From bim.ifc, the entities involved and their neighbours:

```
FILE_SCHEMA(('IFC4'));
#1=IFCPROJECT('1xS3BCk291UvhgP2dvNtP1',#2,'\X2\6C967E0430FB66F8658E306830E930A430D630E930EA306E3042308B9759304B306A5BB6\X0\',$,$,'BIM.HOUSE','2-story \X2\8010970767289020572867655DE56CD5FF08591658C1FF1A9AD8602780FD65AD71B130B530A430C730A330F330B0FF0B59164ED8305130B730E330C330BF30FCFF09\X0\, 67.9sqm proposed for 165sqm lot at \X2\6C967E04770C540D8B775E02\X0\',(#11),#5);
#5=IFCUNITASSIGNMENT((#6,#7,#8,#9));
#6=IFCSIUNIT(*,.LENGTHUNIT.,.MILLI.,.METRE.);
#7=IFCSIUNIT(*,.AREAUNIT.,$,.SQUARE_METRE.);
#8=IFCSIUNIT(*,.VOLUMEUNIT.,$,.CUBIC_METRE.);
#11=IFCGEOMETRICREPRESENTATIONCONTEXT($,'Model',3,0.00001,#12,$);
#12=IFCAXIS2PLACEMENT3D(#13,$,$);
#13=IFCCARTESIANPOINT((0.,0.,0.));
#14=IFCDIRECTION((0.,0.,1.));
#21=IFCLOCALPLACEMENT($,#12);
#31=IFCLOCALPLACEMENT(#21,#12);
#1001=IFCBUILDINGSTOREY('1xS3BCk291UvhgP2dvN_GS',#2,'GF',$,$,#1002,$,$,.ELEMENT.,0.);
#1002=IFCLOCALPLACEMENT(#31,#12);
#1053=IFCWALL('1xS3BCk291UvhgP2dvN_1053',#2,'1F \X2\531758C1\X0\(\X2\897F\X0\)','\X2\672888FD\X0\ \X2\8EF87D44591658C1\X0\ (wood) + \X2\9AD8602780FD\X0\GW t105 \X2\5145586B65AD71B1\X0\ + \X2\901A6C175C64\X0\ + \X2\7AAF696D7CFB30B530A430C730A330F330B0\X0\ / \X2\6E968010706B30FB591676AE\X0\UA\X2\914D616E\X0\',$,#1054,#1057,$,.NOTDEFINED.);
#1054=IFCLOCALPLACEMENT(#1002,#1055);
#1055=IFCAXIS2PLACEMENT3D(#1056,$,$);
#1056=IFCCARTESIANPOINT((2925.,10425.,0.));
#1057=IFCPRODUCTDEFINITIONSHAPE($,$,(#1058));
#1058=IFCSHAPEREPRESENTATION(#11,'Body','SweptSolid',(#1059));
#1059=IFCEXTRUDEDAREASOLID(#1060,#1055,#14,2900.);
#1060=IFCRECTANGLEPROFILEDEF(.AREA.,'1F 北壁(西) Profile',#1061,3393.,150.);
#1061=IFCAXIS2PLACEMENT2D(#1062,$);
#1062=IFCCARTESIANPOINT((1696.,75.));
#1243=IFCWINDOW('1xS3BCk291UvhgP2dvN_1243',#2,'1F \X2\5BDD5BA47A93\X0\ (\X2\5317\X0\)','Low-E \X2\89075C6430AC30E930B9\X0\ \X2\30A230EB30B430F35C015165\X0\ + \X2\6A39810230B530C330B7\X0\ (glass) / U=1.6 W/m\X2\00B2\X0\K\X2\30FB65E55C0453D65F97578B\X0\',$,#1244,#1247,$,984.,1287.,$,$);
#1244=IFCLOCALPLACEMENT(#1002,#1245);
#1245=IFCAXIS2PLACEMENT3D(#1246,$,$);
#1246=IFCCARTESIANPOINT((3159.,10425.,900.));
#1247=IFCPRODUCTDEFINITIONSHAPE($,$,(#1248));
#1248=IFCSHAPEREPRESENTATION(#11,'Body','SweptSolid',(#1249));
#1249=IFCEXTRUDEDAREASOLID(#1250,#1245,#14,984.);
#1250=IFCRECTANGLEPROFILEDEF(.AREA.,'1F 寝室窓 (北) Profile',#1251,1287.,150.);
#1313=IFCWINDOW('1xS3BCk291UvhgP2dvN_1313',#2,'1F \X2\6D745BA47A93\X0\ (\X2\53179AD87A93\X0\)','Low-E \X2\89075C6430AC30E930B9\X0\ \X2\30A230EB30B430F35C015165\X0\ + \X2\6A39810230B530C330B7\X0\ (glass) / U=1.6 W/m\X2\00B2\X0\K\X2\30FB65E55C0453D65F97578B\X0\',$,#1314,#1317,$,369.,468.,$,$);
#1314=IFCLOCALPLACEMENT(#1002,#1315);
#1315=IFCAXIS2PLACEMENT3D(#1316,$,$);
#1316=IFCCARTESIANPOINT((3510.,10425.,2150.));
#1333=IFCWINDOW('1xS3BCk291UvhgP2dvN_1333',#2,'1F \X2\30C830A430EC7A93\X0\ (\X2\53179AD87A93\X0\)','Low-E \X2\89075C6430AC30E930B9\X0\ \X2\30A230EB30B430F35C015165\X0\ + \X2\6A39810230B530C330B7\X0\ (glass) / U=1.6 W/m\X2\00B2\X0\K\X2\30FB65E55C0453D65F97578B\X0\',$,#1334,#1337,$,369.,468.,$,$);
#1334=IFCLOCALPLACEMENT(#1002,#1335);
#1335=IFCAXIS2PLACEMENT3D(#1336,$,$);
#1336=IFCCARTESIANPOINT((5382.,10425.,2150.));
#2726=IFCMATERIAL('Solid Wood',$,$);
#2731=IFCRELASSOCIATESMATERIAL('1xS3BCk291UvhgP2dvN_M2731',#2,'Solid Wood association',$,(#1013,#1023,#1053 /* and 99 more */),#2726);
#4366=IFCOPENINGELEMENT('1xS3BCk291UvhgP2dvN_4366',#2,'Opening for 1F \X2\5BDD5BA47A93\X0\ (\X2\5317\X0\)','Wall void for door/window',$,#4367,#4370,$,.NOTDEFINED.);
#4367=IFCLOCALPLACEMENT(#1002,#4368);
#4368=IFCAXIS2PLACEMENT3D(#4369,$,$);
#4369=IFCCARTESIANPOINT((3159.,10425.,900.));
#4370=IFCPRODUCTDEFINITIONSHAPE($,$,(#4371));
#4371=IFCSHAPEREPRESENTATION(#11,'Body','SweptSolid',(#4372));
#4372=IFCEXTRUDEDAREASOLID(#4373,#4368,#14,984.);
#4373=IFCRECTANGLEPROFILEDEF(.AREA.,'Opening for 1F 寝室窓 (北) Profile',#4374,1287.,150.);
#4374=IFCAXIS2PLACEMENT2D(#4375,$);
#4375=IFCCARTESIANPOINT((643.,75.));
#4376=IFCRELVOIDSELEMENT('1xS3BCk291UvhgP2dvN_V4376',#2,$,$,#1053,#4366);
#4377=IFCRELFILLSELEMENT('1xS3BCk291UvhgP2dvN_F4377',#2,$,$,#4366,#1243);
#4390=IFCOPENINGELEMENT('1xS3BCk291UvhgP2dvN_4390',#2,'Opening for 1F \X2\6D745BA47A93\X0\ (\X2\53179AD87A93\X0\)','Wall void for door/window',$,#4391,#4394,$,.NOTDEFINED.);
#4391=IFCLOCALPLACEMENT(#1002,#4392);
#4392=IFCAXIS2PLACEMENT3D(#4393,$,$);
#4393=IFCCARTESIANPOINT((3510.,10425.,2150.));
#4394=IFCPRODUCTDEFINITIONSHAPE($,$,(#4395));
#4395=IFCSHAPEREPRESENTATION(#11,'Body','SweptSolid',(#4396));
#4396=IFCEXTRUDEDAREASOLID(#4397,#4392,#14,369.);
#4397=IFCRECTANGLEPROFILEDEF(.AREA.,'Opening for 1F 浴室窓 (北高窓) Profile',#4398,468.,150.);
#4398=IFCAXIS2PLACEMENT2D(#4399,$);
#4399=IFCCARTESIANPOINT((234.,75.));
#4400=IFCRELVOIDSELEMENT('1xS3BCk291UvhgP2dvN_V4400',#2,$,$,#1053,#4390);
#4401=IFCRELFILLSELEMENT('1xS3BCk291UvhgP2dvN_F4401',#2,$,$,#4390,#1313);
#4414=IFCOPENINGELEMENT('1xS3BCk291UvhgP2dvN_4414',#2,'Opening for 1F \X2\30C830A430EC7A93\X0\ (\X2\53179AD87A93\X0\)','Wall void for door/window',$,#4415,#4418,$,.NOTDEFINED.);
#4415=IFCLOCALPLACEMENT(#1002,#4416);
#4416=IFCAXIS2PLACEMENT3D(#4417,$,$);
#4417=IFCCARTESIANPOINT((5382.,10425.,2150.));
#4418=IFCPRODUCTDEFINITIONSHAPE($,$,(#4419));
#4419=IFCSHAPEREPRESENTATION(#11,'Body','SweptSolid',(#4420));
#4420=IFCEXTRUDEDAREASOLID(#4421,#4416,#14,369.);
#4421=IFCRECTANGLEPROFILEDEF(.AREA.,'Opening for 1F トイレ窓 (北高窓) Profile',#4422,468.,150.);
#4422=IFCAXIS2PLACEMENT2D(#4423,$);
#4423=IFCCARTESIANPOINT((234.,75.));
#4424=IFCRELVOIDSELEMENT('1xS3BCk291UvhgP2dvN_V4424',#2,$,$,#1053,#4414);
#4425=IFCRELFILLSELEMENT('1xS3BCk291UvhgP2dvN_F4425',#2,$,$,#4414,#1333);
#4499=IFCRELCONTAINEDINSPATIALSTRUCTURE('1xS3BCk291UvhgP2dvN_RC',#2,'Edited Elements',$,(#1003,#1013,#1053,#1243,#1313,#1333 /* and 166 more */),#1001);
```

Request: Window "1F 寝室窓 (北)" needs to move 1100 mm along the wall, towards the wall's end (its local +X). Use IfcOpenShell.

```python
import ifcopenshell
import ifcopenshell.api.geometry
import ifcopenshell.util.placement
import ifcopenshell.util.unit

model = ifcopenshell.open("bim.ifc")
unit_scale = ifcopenshell.util.unit.calculate_unit_scale(model)

window = model.by_id(1243)
opening = window.FillsVoids[0].RelatingOpeningElement
wall = opening.VoidsElements[0].RelatingBuildingElement

wall_matrix = ifcopenshell.util.placement.get_local_placement(wall.ObjectPlacement)
shift = wall_matrix[:3, 0] * 1.1 / unit_scale
before = ifcopenshell.util.placement.get_local_placement(window.ObjectPlacement)[:3, 3].copy()

# The window is not placed relative to its opening, so move both.
for product in (opening, window):
    matrix = ifcopenshell.util.placement.get_local_placement(product.ObjectPlacement)
    matrix[:3, 3] += shift
    ifcopenshell.api.geometry.edit_object_placement(model, product=product, matrix=matrix, is_si=False)

after = ifcopenshell.util.placement.get_local_placement(window.ObjectPlacement)[:3, 3]
print("window moved by", (after - before).round(3) + 0.0)

model.write("bim_rev.ifc")
```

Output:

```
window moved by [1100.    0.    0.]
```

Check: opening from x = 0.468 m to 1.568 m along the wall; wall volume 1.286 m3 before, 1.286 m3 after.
